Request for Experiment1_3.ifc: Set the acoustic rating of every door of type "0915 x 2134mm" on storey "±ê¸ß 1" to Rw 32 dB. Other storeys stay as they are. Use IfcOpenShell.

First a look at what the model holds.

```python
import ifcopenshell
import ifcopenshell.util.element

model = ifcopenshell.open("Experiment1_3.ifc")
print(model.schema)
storey = next(s for s in model.by_type("IfcBuildingStorey") if s.Name == "±ê¸ß 1")
doors = [e for e in ifcopenshell.util.element.get_decomposition(storey) if e.is_a("IfcDoor")]
seen = {}
for e in doors:
    element_type = ifcopenshell.util.element.get_type(e)
    key = (element_type.Name if element_type != e and element_type else None, ifcopenshell.util.element.get_pset(e, "Pset_DoorCommon", "AcousticRating"))
    seen[key] = seen.get(key, 0) + 1
for (name, value), count in sorted(seen.items(), key=str):
    print(count, "x", name, "|", value)
```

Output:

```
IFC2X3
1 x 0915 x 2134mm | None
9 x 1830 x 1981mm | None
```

```python
import ifcopenshell
import ifcopenshell.api.pset
import ifcopenshell.util.element

model = ifcopenshell.open("Experiment1_3.ifc")

storey = next(s for s in model.by_type("IfcBuildingStorey") if s.Name == "±ê¸ß 1")
doors = [e for e in ifcopenshell.util.element.get_decomposition(storey) if e.is_a("IfcDoor")]

count = 0
for e in doors:
    element_type = ifcopenshell.util.element.get_type(e)
    if element_type in (None, e) or element_type.Name != "0915 x 2134mm":
        continue
    # add_pset returns the element's existing set when there is one.
    pset = ifcopenshell.api.pset.add_pset(model, product=e, name="Pset_DoorCommon")
    ifcopenshell.api.pset.edit_pset(model, pset=pset, properties={"AcousticRating": "Rw 32 dB"})
    count += 1

print(count, "doors updated")

model.write("Experiment1_3_v2.ifc")
```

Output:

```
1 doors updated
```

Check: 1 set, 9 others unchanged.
